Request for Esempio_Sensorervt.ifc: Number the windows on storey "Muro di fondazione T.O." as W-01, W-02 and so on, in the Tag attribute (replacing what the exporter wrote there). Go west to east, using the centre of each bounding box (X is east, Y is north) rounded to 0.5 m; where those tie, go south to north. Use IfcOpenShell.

First a look at what the model holds.

```python
import ifcopenshell
import ifcopenshell.util.element
import ifcopenshell.util.placement

model = ifcopenshell.open("Esempio_Sensorervt.ifc")
print(model.schema)
storey = next(s for s in model.by_type("IfcBuildingStorey") if s.Name == "Muro di fondazione T.O.")
windows = [e for e in ifcopenshell.util.element.get_decomposition(storey) if e.is_a("IfcWindow")]
for e in sorted(windows, key=lambda e: e.id()):
    origin = ifcopenshell.util.placement.get_local_placement(e.ObjectPlacement)[:3, 3]
    print(e.id(), e.Tag, e.Name, origin.round(2) + 0.0, sep=" | ")
```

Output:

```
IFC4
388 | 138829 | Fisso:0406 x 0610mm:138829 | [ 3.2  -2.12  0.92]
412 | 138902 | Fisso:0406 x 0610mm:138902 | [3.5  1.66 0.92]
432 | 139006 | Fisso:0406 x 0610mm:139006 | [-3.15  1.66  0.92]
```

```python
import ifcopenshell
import ifcopenshell.geom
import ifcopenshell.util.element
import ifcopenshell.util.shape

model = ifcopenshell.open("Esempio_Sensorervt.ifc")
settings = ifcopenshell.geom.settings()
settings.set("use-world-coords", True)


def centre(element):
    shape = ifcopenshell.geom.create_shape(settings, element)
    return ifcopenshell.util.shape.get_bbox_centroid(shape.geometry)


storey = next(s for s in model.by_type("IfcBuildingStorey") if s.Name == "Muro di fondazione T.O.")
windows = [e for e in ifcopenshell.util.element.get_decomposition(storey) if e.is_a("IfcWindow")]

# Insertion points can sit at a corner or the storey origin, so sort by the geometry (in metres).
centres = {e: centre(e) for e in windows}
windows.sort(key=lambda e: (round(centres[e][0] / 0.5), centres[e][1]))

for i, e in enumerate(windows, start=1):
    number = f"W-{i:02d}"
    e.Tag = number
    print(e.id(), number)

model.write("Esempio_Sensorervt_updated.ifc")
```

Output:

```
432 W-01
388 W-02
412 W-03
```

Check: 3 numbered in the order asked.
